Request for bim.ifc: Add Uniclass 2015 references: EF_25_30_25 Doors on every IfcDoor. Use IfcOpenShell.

First a look at what the model holds.

```python
import ifcopenshell

model = ifcopenshell.open("bim.ifc")
print(model.schema)
print("classifications:", [c.Name for c in model.by_type("IfcClassification")])
for ifc_class in ("IfcDoor", "IfcRoof", "IfcStair", "IfcWall", "IfcWindow"):
    print(ifc_class, len(model.by_type(ifc_class)))
```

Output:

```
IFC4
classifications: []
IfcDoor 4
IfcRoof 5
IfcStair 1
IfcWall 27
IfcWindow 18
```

```python
import ifcopenshell
import ifcopenshell.api.classification

model = ifcopenshell.open("bim.ifc")

system = ifcopenshell.api.classification.add_classification(model, classification="Uniclass 2015")

codes = {
    "IfcDoor": ("EF_25_30_25", "Doors"),
}
for ifc_class, (code, name) in codes.items():
    products = model.by_type(ifc_class)
    ifcopenshell.api.classification.add_reference(
        model, products=products, classification=system, identification=code, name=name
    )
    print(code, len(products))

model.write("bim_rev.ifc")
```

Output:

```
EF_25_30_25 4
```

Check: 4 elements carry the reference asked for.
